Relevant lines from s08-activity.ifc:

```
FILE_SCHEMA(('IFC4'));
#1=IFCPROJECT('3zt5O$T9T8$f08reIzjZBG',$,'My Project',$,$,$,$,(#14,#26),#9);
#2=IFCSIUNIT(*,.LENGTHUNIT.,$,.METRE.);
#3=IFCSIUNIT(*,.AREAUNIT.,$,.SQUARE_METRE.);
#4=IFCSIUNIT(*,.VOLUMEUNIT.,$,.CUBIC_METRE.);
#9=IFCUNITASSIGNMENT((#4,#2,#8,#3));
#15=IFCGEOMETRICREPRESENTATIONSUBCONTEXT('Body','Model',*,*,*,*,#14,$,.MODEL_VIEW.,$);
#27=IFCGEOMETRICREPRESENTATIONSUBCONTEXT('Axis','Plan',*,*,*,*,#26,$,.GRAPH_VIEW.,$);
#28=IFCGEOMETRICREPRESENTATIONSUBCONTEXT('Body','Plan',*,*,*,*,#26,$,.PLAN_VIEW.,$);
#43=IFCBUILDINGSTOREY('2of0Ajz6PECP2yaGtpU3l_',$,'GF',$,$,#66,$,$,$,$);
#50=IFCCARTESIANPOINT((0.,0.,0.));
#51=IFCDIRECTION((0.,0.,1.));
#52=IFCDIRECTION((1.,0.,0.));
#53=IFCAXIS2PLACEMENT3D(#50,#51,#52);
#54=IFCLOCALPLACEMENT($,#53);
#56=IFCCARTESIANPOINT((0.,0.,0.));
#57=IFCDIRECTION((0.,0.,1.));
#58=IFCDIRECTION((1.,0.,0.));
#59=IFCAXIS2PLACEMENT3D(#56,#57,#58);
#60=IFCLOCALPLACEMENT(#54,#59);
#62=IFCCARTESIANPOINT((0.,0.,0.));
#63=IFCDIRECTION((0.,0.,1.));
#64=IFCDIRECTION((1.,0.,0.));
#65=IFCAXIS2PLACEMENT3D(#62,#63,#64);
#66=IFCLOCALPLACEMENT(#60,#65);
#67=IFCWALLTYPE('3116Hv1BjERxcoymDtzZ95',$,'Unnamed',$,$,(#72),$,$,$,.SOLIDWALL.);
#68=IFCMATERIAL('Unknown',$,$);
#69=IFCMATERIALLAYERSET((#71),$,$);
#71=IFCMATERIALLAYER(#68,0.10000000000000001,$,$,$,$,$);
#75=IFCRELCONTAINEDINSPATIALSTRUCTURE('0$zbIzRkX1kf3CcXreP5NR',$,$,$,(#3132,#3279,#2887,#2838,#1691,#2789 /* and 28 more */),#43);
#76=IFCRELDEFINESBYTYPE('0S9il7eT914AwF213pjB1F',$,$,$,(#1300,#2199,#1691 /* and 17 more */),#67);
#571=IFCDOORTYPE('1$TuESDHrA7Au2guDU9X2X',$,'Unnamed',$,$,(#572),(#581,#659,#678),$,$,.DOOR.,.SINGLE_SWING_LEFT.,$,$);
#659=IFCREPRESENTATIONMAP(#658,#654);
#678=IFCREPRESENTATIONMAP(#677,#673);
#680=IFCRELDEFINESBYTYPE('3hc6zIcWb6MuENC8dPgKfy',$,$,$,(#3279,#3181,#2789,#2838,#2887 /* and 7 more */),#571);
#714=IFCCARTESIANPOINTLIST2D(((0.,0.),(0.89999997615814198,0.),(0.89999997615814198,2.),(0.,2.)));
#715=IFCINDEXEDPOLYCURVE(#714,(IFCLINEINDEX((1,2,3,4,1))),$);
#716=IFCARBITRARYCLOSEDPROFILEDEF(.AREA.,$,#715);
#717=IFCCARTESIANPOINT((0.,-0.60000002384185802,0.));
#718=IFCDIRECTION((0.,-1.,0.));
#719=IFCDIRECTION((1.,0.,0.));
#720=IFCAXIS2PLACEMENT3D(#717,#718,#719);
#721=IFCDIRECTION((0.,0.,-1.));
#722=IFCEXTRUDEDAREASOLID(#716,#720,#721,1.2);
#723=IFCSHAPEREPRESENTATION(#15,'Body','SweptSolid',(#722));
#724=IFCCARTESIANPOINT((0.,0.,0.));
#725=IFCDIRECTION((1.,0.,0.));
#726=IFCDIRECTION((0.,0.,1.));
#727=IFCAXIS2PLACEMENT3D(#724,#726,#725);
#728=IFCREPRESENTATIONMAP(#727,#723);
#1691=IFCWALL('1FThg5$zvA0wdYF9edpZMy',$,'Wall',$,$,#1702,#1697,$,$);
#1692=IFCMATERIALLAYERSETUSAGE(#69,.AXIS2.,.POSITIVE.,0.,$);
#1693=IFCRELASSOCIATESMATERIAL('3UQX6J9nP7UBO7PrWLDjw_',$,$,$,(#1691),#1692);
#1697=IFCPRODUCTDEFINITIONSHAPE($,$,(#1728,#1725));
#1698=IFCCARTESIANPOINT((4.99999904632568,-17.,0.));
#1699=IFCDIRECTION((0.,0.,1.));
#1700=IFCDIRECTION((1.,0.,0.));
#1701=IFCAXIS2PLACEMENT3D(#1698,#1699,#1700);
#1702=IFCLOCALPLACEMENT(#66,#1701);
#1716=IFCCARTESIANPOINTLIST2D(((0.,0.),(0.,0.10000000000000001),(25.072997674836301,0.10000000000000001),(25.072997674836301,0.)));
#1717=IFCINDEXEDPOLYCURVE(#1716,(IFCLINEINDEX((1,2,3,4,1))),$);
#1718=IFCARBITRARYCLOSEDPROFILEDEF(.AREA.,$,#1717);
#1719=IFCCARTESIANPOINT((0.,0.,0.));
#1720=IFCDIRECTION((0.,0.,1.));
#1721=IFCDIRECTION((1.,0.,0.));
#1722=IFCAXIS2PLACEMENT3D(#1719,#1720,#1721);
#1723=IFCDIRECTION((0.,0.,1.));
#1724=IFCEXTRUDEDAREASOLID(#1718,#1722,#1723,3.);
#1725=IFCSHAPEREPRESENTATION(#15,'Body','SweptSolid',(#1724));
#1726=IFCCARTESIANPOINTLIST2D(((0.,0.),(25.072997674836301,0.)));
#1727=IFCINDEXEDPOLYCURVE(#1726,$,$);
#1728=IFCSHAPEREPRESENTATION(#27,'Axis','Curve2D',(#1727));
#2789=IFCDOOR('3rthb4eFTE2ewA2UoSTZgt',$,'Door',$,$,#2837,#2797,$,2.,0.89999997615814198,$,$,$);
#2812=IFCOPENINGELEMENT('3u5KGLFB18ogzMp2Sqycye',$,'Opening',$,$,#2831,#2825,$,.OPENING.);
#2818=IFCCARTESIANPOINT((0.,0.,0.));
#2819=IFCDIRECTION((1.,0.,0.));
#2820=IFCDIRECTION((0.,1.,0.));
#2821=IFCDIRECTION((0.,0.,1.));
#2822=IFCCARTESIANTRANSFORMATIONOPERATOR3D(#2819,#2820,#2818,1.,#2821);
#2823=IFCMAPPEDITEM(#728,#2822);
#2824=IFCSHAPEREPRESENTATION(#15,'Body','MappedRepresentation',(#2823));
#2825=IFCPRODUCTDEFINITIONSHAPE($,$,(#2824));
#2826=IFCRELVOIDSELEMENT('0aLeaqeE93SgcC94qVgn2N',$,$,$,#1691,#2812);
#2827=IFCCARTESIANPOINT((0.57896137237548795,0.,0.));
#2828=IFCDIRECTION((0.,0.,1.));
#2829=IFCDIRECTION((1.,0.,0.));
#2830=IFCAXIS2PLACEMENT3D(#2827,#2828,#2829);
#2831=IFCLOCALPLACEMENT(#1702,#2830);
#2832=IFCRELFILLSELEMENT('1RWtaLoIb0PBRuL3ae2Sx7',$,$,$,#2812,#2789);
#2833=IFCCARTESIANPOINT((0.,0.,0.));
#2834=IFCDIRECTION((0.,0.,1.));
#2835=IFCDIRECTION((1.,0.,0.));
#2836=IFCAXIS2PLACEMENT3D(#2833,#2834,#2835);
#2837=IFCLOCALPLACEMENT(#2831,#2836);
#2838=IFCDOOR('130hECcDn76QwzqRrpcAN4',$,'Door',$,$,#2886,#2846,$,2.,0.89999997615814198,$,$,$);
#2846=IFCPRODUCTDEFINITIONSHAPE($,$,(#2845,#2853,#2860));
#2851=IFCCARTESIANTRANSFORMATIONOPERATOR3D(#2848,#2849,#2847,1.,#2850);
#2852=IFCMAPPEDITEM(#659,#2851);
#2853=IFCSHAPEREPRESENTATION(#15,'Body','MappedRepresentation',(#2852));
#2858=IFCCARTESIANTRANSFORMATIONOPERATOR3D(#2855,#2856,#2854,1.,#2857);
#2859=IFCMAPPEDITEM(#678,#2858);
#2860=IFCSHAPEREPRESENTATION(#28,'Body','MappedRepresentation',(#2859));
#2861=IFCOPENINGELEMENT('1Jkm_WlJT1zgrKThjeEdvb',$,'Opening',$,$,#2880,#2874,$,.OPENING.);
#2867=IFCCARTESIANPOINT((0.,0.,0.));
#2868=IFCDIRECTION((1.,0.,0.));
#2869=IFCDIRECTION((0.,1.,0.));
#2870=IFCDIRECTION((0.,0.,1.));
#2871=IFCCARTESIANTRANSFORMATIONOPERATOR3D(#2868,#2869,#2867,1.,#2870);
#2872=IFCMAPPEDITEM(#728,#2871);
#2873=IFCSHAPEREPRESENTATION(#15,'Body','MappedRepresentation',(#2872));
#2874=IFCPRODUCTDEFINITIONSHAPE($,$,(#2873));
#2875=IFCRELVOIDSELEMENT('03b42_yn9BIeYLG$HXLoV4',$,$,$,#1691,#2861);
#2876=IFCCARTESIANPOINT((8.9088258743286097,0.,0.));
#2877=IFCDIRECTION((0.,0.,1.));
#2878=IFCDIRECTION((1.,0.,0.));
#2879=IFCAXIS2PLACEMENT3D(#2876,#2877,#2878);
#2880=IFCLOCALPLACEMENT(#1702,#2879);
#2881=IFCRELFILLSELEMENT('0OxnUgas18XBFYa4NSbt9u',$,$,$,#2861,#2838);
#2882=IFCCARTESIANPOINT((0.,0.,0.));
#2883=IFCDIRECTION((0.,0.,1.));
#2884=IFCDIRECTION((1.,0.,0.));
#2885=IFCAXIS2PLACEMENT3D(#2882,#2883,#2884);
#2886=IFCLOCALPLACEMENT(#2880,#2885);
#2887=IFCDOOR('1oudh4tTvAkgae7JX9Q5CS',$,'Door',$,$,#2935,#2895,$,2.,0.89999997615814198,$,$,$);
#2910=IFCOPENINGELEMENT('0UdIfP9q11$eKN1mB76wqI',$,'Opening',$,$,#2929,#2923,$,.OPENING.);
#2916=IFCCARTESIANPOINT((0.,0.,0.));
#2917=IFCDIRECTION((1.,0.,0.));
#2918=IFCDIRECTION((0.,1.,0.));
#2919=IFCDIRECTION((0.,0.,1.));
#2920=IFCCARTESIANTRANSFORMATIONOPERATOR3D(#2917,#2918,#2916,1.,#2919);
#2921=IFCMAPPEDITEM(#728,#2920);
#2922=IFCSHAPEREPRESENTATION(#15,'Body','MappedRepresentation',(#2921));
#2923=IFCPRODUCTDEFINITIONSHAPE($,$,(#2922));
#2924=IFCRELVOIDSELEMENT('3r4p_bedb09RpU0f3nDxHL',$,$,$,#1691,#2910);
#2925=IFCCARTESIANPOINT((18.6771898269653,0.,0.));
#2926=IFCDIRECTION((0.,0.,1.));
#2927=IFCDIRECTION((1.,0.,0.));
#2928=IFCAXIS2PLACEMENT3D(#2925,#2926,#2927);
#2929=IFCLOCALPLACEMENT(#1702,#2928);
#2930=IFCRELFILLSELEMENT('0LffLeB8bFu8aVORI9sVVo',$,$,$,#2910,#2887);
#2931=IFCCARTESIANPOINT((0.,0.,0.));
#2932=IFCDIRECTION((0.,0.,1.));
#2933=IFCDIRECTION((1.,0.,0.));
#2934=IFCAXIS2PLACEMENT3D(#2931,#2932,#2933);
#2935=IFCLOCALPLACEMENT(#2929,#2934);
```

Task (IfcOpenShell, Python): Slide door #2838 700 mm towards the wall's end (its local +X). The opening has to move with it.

```python
import ifcopenshell
import ifcopenshell.api.geometry
import ifcopenshell.util.placement

model = ifcopenshell.open("s08-activity.ifc")

door = model.by_guid("130hECcDn76QwzqRrpcAN4")
opening = door.FillsVoids[0].RelatingOpeningElement
wall = opening.VoidsElements[0].RelatingBuildingElement

wall_matrix = ifcopenshell.util.placement.get_local_placement(wall.ObjectPlacement)
shift = wall_matrix[:3, 0] * 0.7
before = ifcopenshell.util.placement.get_local_placement(door.ObjectPlacement)[:3, 3].copy()

# The door is placed relative to its opening, so it follows when the opening moves.
matrix = ifcopenshell.util.placement.get_local_placement(opening.ObjectPlacement)
matrix[:3, 3] += shift
ifcopenshell.api.geometry.edit_object_placement(
    model, product=opening, matrix=matrix, is_si=False, should_transform_children=True
)

after = ifcopenshell.util.placement.get_local_placement(door.ObjectPlacement)[:3, 3]
print("door moved by", (after - before).round(3) + 0.0)

model.write("s08-activity_edited.ifc")
```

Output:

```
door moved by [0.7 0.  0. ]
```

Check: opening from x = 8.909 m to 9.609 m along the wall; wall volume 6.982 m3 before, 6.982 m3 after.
